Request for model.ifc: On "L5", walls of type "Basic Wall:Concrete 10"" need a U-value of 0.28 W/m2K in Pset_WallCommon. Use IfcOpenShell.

First a look at what the model holds.

```python
import ifcopenshell
import ifcopenshell.util.element

model = ifcopenshell.open("model.ifc")
print(model.schema)
storey = next(s for s in model.by_type("IfcBuildingStorey") if s.Name == "L5")
walls = [e for e in ifcopenshell.util.element.get_decomposition(storey) if e.is_a("IfcWall")]
seen = {}
for e in walls:
    element_type = ifcopenshell.util.element.get_type(e)
    key = (element_type.Name if element_type != e and element_type else None, ifcopenshell.util.element.get_pset(e, "Pset_WallCommon", "ThermalTransmittance"))
    seen[key] = seen.get(key, 0) + 1
for (name, value), count in sorted(seen.items(), key=str):
    print(count, "x", name, "|", value)
```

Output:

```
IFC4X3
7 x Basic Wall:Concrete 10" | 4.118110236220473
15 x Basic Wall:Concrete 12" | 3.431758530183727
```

```python
import ifcopenshell
import ifcopenshell.api.pset
import ifcopenshell.util.element

model = ifcopenshell.open("model.ifc")

storey = next(s for s in model.by_type("IfcBuildingStorey") if s.Name == "L5")
walls = [e for e in ifcopenshell.util.element.get_decomposition(storey) if e.is_a("IfcWall")]

count = 0
for e in walls:
    element_type = ifcopenshell.util.element.get_type(e)
    if element_type in (None, e) or element_type.Name != 'Basic Wall:Concrete 10"':
        continue
    # add_pset returns the element's existing set when there is one.
    pset = ifcopenshell.api.pset.add_pset(model, product=e, name="Pset_WallCommon")
    ifcopenshell.api.pset.edit_pset(model, pset=pset, properties={"ThermalTransmittance": 0.28})
    count += 1

print(count, "walls updated")

model.write("model_updated.ifc")
```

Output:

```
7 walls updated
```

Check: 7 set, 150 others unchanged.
